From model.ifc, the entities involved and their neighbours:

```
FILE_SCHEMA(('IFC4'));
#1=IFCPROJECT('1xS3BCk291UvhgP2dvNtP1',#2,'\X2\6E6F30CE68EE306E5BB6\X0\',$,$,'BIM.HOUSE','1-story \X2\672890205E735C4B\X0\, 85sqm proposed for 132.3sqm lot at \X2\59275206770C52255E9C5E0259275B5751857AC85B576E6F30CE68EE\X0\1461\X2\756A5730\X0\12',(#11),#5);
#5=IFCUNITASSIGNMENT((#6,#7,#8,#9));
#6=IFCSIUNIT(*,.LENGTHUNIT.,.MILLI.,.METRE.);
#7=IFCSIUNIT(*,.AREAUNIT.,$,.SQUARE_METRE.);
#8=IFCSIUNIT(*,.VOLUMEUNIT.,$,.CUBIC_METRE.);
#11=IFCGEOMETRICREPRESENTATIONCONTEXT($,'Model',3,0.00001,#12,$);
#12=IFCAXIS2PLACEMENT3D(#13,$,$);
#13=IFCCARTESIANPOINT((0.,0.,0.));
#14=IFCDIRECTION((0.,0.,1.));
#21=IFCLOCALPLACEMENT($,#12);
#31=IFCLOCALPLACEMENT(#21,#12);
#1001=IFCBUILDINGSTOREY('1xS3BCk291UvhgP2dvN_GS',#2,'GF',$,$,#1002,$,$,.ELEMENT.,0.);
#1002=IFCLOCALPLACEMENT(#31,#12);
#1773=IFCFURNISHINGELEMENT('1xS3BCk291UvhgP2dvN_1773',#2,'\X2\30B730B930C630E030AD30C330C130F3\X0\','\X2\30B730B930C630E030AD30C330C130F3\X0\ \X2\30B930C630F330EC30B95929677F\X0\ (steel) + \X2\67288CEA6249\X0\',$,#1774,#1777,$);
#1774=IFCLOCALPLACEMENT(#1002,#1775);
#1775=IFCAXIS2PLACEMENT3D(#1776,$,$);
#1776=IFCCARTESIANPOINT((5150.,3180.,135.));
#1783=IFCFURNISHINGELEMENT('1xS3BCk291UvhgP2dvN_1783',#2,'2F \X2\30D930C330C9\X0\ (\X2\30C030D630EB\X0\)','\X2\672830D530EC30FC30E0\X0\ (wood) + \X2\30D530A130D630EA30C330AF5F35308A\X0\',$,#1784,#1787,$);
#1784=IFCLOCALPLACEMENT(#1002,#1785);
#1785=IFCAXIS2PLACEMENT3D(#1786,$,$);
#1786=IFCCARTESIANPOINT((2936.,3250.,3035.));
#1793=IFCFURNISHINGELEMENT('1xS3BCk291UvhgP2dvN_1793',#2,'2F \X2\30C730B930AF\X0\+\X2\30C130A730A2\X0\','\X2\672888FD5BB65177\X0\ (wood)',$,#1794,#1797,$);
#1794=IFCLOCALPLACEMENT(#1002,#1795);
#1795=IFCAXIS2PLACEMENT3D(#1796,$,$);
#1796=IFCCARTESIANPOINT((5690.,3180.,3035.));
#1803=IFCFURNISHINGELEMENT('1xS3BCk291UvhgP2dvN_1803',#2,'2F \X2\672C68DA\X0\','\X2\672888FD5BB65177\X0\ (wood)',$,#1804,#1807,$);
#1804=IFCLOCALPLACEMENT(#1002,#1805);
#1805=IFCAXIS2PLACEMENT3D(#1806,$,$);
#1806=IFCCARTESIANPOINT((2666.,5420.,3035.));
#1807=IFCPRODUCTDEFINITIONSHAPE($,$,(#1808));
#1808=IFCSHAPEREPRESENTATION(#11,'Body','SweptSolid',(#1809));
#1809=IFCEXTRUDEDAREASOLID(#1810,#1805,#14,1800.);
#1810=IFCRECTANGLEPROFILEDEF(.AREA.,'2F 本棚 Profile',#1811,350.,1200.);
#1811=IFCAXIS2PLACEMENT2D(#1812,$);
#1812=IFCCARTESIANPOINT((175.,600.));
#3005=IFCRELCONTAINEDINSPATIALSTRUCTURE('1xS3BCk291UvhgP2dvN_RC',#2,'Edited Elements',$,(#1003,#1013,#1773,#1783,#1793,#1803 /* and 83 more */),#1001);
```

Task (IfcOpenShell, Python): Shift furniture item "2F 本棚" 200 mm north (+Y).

```python
import ifcopenshell
import ifcopenshell.api.geometry
import ifcopenshell.util.placement

model = ifcopenshell.open("model.ifc")

item = model.by_guid("1xS3BCk291UvhgP2dvN_1803")
matrix = ifcopenshell.util.placement.get_local_placement(item.ObjectPlacement)
matrix[1, 3] += 200.0
ifcopenshell.api.geometry.edit_object_placement(model, product=item, matrix=matrix, is_si=False)

print(ifcopenshell.util.placement.get_local_placement(item.ObjectPlacement).round(3) + 0.0)

model.write("model_edited.ifc")
```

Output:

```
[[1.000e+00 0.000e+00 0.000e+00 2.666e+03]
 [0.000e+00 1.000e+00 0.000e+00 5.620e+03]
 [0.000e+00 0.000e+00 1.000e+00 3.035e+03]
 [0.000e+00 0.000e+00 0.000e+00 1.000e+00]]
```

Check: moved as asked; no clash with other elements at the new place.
